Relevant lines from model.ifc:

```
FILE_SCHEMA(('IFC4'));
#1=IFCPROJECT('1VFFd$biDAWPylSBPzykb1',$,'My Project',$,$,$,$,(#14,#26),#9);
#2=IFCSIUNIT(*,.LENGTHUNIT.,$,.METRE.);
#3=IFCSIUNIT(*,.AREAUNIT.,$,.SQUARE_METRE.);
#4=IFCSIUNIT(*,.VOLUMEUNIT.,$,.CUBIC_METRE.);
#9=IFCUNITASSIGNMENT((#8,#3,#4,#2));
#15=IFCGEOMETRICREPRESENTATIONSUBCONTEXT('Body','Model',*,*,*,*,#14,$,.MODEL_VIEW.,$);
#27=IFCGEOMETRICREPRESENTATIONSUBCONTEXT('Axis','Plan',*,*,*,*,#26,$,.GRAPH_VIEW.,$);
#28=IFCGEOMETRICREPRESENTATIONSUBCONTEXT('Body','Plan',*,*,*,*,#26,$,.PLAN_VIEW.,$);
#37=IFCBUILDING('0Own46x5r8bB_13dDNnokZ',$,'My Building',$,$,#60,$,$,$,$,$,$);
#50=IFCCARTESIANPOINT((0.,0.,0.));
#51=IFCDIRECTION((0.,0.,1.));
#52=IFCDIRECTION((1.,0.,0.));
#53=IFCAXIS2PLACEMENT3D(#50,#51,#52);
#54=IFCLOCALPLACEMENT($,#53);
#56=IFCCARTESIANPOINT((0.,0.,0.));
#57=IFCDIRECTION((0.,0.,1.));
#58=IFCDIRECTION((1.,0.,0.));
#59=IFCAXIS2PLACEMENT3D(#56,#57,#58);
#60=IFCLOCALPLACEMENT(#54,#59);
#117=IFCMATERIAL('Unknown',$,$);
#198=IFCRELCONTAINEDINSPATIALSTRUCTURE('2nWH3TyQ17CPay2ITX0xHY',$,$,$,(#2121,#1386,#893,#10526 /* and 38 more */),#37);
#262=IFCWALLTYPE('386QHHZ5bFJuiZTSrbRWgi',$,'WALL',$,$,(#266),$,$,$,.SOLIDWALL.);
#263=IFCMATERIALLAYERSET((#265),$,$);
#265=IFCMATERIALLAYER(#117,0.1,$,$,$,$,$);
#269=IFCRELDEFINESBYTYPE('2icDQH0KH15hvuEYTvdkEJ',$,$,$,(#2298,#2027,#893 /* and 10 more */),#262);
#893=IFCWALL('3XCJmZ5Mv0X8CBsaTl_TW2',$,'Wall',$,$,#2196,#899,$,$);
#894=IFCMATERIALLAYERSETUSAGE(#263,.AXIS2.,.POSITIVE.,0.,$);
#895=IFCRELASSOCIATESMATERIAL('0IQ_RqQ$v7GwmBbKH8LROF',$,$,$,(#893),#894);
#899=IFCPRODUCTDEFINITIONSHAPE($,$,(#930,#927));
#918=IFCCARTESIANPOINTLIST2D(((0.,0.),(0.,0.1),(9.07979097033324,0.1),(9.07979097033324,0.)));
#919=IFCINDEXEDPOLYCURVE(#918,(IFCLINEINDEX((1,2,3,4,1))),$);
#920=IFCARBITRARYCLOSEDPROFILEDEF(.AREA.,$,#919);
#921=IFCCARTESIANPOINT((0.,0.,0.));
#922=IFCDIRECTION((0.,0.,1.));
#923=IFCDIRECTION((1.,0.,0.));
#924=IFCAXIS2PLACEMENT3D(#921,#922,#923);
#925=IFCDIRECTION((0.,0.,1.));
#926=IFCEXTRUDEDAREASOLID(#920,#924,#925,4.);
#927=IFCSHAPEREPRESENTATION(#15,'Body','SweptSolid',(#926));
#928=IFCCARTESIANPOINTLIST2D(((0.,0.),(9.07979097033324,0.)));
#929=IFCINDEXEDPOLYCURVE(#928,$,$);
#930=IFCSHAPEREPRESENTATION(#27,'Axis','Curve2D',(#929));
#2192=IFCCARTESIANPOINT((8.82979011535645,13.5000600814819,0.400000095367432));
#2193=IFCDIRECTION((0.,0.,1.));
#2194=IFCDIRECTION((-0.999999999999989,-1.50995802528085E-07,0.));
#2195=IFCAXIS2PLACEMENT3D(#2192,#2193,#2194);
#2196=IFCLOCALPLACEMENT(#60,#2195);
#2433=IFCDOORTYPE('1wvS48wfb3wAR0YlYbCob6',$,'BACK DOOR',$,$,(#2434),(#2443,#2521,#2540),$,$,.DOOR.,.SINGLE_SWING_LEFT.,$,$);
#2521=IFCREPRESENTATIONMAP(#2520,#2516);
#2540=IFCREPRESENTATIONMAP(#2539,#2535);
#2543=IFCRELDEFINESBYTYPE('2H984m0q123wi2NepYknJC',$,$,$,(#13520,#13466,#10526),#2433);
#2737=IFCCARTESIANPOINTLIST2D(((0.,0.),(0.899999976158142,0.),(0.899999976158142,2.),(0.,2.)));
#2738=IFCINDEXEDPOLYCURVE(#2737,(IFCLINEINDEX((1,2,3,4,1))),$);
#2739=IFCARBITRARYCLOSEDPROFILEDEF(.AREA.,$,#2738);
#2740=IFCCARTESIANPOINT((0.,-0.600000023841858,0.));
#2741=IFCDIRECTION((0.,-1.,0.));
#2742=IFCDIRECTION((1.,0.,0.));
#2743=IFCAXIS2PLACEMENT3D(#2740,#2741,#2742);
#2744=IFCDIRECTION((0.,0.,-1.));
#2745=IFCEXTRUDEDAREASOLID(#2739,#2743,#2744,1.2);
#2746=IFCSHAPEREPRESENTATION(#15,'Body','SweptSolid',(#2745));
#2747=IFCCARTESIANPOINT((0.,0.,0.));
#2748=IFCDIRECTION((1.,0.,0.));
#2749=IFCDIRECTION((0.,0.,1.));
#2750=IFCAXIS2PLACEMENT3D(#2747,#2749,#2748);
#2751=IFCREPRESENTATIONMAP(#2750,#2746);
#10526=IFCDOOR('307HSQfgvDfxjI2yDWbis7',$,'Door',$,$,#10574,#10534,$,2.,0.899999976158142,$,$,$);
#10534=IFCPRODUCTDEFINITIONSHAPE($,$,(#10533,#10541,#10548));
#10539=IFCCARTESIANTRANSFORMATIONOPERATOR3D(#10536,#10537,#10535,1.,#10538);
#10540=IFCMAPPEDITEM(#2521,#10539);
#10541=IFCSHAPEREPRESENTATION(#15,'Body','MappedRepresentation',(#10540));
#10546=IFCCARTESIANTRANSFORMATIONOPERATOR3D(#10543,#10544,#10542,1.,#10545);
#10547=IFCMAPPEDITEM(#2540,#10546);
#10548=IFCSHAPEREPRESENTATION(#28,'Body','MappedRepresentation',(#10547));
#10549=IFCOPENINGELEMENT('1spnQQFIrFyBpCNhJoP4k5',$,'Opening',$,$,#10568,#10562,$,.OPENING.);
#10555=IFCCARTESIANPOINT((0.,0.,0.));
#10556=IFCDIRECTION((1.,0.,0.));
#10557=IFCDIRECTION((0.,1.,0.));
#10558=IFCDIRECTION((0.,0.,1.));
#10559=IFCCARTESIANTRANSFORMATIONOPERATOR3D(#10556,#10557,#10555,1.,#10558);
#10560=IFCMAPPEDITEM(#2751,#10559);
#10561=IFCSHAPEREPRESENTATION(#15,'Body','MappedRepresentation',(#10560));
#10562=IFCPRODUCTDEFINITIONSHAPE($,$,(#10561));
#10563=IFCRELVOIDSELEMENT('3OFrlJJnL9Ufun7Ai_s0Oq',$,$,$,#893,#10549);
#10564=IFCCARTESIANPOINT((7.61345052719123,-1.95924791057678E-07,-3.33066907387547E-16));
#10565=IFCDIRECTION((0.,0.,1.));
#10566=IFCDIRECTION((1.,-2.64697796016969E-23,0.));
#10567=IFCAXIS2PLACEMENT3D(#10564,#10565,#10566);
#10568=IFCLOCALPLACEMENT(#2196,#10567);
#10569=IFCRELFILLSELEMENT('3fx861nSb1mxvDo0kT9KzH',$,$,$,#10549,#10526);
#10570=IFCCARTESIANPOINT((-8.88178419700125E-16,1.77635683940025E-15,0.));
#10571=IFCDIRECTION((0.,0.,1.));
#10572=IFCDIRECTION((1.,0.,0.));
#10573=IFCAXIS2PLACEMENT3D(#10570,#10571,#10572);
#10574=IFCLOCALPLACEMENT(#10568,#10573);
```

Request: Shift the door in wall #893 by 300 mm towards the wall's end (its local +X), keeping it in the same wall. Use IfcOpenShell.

```python
import ifcopenshell
import ifcopenshell.api.geometry
import ifcopenshell.util.placement
import ifcopenshell.util.unit

model = ifcopenshell.open("model.ifc")
unit_scale = ifcopenshell.util.unit.calculate_unit_scale(model)

door = model.by_guid("307HSQfgvDfxjI2yDWbis7")
opening = door.FillsVoids[0].RelatingOpeningElement
wall = opening.VoidsElements[0].RelatingBuildingElement

wall_matrix = ifcopenshell.util.placement.get_local_placement(wall.ObjectPlacement)
shift = wall_matrix[:3, 0] * 0.3 / unit_scale
before = ifcopenshell.util.placement.get_local_placement(door.ObjectPlacement)[:3, 3].copy()

# The door is placed relative to its opening, so it follows when the opening moves.
matrix = ifcopenshell.util.placement.get_local_placement(opening.ObjectPlacement)
matrix[:3, 3] += shift
ifcopenshell.api.geometry.edit_object_placement(
    model, product=opening, matrix=matrix, is_si=False, should_transform_children=True
)

after = ifcopenshell.util.placement.get_local_placement(door.ObjectPlacement)[:3, 3]
print("door moved by", (after - before).round(3) + 0.0)

model.write("model-out.ifc")
```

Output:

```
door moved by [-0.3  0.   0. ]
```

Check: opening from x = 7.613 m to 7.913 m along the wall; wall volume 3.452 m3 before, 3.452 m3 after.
